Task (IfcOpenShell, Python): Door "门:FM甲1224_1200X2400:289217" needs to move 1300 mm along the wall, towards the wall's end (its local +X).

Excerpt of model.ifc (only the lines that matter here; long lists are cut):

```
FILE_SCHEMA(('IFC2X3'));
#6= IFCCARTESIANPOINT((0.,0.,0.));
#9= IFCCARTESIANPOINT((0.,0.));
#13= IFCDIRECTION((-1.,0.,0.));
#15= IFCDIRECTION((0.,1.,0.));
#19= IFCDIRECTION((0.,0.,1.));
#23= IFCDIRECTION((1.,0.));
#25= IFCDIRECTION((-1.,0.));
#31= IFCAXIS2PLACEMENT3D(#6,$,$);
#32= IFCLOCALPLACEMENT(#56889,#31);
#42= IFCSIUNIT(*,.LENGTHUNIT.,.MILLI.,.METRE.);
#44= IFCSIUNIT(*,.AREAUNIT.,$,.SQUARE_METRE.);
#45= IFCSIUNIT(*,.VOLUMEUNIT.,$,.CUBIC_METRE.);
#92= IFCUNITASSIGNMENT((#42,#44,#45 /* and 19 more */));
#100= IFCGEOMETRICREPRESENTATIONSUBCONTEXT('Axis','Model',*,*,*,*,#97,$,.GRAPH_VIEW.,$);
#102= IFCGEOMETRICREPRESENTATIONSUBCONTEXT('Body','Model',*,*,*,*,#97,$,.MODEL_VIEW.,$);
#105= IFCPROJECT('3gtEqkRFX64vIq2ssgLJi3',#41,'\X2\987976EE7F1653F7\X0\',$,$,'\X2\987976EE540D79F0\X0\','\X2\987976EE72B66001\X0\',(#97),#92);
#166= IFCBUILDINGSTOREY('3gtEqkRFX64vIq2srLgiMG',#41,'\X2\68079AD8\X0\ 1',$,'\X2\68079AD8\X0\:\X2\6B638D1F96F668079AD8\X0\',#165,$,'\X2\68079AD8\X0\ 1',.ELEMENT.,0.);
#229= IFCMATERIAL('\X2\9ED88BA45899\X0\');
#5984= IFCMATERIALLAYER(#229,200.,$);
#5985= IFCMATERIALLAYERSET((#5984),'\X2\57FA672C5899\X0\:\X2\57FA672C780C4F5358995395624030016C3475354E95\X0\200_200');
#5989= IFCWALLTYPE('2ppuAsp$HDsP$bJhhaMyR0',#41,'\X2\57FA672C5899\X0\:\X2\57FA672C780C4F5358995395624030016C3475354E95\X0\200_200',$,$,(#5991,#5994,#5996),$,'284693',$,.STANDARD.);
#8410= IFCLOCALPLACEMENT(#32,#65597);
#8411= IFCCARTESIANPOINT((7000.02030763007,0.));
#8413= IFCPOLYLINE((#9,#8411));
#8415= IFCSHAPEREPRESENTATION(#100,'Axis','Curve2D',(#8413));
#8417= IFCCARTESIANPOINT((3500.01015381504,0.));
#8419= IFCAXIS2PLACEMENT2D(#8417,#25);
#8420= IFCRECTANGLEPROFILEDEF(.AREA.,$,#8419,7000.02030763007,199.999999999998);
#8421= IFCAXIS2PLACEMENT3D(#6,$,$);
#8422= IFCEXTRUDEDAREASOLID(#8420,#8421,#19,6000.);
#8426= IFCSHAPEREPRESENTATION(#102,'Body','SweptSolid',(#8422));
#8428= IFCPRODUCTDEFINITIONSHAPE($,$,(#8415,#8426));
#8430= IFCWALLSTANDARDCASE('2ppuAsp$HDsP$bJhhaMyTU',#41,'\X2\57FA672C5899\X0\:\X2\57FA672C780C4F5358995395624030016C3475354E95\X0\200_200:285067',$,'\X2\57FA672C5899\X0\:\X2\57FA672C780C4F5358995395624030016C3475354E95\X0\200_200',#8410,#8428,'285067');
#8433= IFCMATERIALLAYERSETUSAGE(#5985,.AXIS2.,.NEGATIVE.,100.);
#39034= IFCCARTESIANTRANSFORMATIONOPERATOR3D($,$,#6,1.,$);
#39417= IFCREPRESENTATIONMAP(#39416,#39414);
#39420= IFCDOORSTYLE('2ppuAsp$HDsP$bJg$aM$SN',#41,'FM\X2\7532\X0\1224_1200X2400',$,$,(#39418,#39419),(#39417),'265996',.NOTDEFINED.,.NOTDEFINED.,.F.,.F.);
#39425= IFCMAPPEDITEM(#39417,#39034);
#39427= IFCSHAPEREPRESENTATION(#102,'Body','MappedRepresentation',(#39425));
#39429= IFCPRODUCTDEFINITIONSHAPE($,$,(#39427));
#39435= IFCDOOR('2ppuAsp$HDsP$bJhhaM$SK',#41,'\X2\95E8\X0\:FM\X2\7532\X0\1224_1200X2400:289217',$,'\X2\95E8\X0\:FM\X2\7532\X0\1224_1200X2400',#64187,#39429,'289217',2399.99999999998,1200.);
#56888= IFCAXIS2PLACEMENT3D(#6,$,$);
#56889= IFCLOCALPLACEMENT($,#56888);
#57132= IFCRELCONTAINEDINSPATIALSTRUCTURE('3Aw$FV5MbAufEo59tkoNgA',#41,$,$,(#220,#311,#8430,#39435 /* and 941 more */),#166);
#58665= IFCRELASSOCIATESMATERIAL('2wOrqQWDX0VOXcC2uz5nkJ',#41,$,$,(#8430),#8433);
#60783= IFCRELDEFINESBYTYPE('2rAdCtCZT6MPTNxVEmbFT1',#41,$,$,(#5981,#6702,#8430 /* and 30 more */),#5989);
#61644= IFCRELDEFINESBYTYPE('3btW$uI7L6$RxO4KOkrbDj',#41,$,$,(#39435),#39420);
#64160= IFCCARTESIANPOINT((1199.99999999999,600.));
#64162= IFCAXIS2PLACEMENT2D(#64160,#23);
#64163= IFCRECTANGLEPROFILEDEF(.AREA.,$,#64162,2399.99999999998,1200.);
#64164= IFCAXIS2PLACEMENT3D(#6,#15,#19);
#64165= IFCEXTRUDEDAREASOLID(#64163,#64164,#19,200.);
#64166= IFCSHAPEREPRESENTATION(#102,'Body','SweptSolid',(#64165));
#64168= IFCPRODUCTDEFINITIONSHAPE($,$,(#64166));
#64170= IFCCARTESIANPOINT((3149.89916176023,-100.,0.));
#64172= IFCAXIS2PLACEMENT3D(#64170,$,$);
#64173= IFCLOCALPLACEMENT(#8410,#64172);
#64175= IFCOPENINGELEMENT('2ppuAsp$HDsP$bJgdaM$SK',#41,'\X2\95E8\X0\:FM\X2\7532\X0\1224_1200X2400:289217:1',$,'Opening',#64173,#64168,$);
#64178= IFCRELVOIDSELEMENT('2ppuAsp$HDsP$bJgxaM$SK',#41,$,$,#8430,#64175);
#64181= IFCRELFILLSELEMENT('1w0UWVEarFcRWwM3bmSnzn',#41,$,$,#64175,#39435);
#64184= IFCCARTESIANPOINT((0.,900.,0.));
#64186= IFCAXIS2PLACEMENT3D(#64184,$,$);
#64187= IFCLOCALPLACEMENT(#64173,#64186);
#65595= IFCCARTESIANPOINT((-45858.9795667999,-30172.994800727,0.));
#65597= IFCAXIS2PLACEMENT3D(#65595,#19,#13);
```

```python
import ifcopenshell
import ifcopenshell.api.geometry
import ifcopenshell.util.placement
import ifcopenshell.util.unit

model = ifcopenshell.open("model.ifc")
unit_scale = ifcopenshell.util.unit.calculate_unit_scale(model)

door = model.by_guid("2ppuAsp$HDsP$bJhhaM$SK")
opening = door.FillsVoids[0].RelatingOpeningElement
wall = opening.VoidsElements[0].RelatingBuildingElement

wall_matrix = ifcopenshell.util.placement.get_local_placement(wall.ObjectPlacement)
shift = wall_matrix[:3, 0] * 1.3 / unit_scale
before = ifcopenshell.util.placement.get_local_placement(door.ObjectPlacement)[:3, 3].copy()

# The door is placed relative to its opening, so it follows when the opening moves.
matrix = ifcopenshell.util.placement.get_local_placement(opening.ObjectPlacement)
matrix[:3, 3] += shift
ifcopenshell.api.geometry.edit_object_placement(
    model, product=opening, matrix=matrix, is_si=False, should_transform_children=True
)

after = ifcopenshell.util.placement.get_local_placement(door.ObjectPlacement)[:3, 3]
print("door moved by", (after - before).round(3) + 0.0)

model.write("model_updated.ifc")
```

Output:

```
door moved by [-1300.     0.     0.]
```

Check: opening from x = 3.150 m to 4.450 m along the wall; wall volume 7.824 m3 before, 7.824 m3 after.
